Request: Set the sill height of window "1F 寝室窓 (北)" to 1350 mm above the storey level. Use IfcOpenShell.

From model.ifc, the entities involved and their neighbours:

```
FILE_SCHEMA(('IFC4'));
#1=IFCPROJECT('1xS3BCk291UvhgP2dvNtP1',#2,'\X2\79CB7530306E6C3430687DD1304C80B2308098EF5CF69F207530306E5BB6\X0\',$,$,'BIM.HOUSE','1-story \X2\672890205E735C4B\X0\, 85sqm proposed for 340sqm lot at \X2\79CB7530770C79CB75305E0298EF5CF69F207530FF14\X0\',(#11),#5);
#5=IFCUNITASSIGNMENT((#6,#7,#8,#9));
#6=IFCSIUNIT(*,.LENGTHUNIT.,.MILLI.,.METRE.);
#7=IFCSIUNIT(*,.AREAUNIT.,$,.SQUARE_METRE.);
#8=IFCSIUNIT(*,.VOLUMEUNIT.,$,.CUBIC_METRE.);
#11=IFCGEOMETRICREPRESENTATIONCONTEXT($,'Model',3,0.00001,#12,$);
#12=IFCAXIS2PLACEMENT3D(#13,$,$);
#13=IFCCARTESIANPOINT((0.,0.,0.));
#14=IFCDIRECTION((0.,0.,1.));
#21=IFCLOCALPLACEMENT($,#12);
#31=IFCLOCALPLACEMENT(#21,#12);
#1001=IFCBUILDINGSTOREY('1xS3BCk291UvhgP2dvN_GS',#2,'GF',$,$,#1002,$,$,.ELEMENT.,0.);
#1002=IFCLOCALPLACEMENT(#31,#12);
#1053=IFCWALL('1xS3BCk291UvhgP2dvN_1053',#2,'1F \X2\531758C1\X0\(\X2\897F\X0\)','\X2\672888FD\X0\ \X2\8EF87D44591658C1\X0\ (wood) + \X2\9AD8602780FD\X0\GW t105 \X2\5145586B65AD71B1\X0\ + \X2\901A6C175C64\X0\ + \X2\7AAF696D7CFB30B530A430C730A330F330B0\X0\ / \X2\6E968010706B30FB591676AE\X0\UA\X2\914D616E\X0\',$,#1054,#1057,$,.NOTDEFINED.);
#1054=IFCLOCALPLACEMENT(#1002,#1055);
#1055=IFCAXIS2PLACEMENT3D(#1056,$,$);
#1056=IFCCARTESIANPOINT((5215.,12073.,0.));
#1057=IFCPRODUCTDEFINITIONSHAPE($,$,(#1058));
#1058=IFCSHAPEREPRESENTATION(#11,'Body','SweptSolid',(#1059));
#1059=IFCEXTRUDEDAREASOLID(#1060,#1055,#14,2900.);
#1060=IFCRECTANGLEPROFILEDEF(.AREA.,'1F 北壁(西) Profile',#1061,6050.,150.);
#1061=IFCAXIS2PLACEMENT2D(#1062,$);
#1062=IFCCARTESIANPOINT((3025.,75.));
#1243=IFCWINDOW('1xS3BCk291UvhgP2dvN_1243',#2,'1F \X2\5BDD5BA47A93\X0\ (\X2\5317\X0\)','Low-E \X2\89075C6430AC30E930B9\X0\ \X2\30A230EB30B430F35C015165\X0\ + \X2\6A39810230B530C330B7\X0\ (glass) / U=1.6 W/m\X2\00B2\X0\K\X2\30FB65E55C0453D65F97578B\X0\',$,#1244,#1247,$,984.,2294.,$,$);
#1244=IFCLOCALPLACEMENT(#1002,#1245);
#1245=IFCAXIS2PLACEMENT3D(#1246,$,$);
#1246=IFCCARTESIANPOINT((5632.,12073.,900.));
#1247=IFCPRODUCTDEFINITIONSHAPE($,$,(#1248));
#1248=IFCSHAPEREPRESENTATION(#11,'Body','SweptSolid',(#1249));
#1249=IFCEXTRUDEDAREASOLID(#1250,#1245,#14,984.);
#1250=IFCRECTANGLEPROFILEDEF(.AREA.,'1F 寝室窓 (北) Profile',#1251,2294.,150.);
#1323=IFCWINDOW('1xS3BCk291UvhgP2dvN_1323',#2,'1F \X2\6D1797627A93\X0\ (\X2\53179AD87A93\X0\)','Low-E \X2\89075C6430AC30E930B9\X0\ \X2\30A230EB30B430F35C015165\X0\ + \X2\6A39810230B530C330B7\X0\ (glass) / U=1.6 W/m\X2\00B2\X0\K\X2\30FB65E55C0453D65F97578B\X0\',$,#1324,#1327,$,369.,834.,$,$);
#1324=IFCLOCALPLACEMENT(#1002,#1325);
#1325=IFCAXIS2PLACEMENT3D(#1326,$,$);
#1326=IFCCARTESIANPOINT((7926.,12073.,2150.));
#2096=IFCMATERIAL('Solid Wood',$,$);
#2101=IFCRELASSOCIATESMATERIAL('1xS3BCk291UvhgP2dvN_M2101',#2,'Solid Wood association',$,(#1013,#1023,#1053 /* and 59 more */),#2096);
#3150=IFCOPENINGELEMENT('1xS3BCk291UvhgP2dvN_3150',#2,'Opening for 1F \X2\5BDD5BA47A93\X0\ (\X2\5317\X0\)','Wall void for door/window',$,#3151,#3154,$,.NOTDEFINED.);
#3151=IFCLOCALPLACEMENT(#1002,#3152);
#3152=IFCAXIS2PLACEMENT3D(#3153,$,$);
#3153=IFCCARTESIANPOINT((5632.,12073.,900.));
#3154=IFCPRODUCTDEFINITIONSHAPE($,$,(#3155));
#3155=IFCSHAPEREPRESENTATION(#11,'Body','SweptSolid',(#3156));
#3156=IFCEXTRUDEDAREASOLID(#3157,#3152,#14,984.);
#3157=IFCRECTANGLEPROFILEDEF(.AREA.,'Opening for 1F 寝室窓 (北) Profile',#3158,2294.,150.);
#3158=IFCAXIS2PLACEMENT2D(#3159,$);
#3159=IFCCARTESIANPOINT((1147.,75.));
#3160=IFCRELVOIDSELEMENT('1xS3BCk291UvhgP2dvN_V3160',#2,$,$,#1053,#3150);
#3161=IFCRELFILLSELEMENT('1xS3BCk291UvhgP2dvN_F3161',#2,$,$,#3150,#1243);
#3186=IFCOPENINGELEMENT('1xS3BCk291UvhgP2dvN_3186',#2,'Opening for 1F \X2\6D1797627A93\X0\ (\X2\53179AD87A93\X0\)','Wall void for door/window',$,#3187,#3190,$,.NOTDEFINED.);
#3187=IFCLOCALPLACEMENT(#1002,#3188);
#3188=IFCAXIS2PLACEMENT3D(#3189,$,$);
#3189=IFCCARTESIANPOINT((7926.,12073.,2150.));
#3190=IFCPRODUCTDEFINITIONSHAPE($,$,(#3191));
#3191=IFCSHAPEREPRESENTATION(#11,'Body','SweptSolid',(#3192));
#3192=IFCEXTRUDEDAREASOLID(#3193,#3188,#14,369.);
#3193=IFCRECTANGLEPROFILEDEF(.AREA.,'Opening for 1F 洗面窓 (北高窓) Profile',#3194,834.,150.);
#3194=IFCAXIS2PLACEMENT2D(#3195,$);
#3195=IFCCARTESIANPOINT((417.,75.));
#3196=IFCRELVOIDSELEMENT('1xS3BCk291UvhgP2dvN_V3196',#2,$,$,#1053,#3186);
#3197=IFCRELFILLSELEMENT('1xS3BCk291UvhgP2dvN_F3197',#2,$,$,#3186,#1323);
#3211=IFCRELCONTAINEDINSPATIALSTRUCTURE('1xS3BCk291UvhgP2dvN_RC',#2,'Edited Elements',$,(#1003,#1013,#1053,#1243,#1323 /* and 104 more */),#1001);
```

```python
import numpy as np
import ifcopenshell
import ifcopenshell.api.geometry
import ifcopenshell.geom
import ifcopenshell.util.element
import ifcopenshell.util.placement
import ifcopenshell.util.shape
import ifcopenshell.util.unit

model = ifcopenshell.open("model.ifc")
unit_scale = ifcopenshell.util.unit.calculate_unit_scale(model)

window = model.by_guid("1xS3BCk291UvhgP2dvN_1243")
opening = window.FillsVoids[0].RelatingOpeningElement
storey = ifcopenshell.util.element.get_container(window, ifc_class="IfcBuildingStorey")
level = ifcopenshell.util.placement.get_local_placement(storey.ObjectPlacement)[2, 3]

# The opening's origin need not be at the sill, so measure its lowest point.
shape = ifcopenshell.geom.create_shape(ifcopenshell.geom.settings(), opening)
bottom = ifcopenshell.util.shape.get_shape_bottom_elevation(shape, shape.geometry) / unit_scale
dz = level + 1.35 / unit_scale - bottom

shift = np.array([0.0, 0.0, dz])
# The window is not placed relative to its opening, so move both.
for product in (opening, window):
    matrix = ifcopenshell.util.placement.get_local_placement(product.ObjectPlacement)
    matrix[:3, 3] += shift
    ifcopenshell.api.geometry.edit_object_placement(model, product=product, matrix=matrix, is_si=False)

print(f"moved by {dz * unit_scale:+.3f} m")

model.write("model-out.ifc")
```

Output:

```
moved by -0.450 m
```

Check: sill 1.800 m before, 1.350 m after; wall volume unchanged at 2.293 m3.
